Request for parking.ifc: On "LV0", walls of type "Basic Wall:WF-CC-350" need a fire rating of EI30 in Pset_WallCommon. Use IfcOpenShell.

First a look at what the model holds.

```python
import ifcopenshell
import ifcopenshell.util.element

model = ifcopenshell.open("parking.ifc")
print(model.schema)
storey = next(s for s in model.by_type("IfcBuildingStorey") if s.Name == "LV0")
walls = [e for e in ifcopenshell.util.element.get_decomposition(storey) if e.is_a("IfcWall")]
seen = {}
for e in walls:
    element_type = ifcopenshell.util.element.get_type(e)
    key = (element_type.Name if element_type != e and element_type else None, ifcopenshell.util.element.get_pset(e, "Pset_WallCommon", "FireRating"))
    seen[key] = seen.get(key, 0) + 1
for (name, value), count in sorted(seen.items(), key=str):
    print(count, "x", name, "|", value)
```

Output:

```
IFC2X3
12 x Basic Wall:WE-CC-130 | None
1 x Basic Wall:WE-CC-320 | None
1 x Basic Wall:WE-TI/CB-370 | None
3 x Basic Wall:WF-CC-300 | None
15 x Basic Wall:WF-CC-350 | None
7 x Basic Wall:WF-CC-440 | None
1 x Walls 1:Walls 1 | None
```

```python
import ifcopenshell
import ifcopenshell.api.pset
import ifcopenshell.util.element

model = ifcopenshell.open("parking.ifc")

storey = next(s for s in model.by_type("IfcBuildingStorey") if s.Name == "LV0")
walls = [e for e in ifcopenshell.util.element.get_decomposition(storey) if e.is_a("IfcWall")]

count = 0
for e in walls:
    element_type = ifcopenshell.util.element.get_type(e)
    if element_type in (None, e) or element_type.Name != "Basic Wall:WF-CC-350":
        continue
    # add_pset returns the element's existing set when there is one.
    pset = ifcopenshell.api.pset.add_pset(model, product=e, name="Pset_WallCommon")
    ifcopenshell.api.pset.edit_pset(model, pset=pset, properties={"FireRating": "EI30"})
    count += 1

print(count, "walls updated")

model.write("parking_v2.ifc")
```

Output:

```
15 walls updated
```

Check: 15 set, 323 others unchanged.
